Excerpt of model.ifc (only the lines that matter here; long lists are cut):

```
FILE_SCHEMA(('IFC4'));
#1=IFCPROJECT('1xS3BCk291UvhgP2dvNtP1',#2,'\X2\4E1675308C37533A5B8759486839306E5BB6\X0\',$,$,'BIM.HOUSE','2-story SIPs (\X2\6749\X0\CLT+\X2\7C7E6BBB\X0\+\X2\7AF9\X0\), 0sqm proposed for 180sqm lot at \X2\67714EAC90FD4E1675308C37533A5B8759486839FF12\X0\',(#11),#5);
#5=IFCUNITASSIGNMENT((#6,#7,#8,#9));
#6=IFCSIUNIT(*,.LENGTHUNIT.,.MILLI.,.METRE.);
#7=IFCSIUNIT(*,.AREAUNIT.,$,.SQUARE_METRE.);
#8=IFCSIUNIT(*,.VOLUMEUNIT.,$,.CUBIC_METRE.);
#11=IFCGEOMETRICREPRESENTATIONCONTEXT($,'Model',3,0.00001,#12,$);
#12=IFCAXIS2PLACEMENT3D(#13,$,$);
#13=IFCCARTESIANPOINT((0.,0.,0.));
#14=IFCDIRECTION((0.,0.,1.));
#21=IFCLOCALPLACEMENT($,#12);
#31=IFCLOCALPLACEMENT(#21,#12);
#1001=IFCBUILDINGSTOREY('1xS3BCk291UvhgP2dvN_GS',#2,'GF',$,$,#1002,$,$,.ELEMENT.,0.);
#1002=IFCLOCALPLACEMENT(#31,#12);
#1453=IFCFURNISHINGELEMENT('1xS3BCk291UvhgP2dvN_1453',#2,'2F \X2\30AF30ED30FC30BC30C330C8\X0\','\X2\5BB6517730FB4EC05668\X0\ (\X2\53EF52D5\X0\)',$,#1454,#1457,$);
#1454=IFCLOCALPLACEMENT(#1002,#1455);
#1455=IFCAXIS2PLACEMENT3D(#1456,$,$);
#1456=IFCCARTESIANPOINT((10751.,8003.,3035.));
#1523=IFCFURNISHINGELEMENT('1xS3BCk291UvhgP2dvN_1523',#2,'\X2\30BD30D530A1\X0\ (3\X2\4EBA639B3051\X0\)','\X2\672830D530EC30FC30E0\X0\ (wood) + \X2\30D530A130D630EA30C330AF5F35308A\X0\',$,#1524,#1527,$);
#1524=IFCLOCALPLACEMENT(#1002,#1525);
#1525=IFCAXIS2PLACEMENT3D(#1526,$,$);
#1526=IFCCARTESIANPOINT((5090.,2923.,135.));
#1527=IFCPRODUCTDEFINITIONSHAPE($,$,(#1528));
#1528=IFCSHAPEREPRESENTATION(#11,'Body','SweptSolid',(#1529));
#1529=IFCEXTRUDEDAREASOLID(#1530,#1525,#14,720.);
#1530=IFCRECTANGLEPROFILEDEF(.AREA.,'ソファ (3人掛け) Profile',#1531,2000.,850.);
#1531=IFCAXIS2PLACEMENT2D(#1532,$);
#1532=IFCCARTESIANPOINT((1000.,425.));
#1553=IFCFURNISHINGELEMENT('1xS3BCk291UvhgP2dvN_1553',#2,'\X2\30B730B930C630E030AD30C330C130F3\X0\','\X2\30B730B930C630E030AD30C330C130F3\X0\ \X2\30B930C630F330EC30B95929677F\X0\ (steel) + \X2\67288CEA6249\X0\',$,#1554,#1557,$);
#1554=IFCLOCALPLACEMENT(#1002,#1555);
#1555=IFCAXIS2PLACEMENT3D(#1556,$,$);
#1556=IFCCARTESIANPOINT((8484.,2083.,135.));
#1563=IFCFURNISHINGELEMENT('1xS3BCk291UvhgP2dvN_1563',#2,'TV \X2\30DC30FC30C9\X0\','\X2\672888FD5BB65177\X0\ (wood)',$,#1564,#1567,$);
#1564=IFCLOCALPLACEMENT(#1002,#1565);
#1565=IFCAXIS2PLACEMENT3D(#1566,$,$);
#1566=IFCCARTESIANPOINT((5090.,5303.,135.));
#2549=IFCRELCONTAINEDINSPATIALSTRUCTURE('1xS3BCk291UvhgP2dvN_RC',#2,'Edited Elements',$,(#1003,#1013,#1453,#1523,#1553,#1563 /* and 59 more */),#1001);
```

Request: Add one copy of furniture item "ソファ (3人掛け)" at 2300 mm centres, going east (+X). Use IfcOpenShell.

```python
import numpy as np
import ifcopenshell
import ifcopenshell.api.geometry
import ifcopenshell.api.root
import ifcopenshell.util.element
import ifcopenshell.util.placement
import ifcopenshell.util.unit

model = ifcopenshell.open("model.ifc")
unit_scale = ifcopenshell.util.unit.calculate_unit_scale(model)


def reuse_history(source, copy):
    """copy_class also copies each property set's owner history, people and application; keep the originals."""
    for rel in copy.IsDefinedBy:
        if rel.is_a("IfcRelDefinesByProperties") and (history := rel.RelatingPropertyDefinition.OwnerHistory):
            rel.RelatingPropertyDefinition.OwnerHistory = source.OwnerHistory
            ifcopenshell.util.element.remove_deep2(model, history)


source = model.by_guid("1xS3BCk291UvhgP2dvN_1523")
base = ifcopenshell.util.placement.get_local_placement(source.ObjectPlacement)
step = np.array([1.0, 0.0, 0.0]) * 2.3 / unit_scale

for i in range(1, 2):
    copy = ifcopenshell.api.root.copy_class(model, product=source)
    copy.Representation = ifcopenshell.util.element.copy_deep(
        model, source.Representation, exclude=["IfcGeometricRepresentationContext", "IfcRepresentationMap"]
    )
    reuse_history(source, copy)
    matrix = base.copy()
    matrix[:3, 3] += i * step
    print("added at", matrix[:3, 3].round(3) + 0.0)
    ifcopenshell.api.geometry.edit_object_placement(model, product=copy, matrix=matrix, is_si=False)

model.write("model-out.ifc")
```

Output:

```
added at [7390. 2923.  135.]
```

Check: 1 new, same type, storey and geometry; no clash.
